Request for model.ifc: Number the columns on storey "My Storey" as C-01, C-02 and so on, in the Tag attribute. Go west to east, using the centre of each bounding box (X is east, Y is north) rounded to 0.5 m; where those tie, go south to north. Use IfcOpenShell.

First a look at what the model holds.

```python
import ifcopenshell
import ifcopenshell.util.element
import ifcopenshell.util.placement

model = ifcopenshell.open("model.ifc")
print(model.schema)
storey = next(s for s in model.by_type("IfcBuildingStorey") if s.Name == "My Storey")
columns = [e for e in ifcopenshell.util.element.get_decomposition(storey) if e.is_a("IfcColumn")]
for e in sorted(columns, key=lambda e: e.id()):
    origin = ifcopenshell.util.placement.get_local_placement(e.ObjectPlacement)[:3, 3]
    print(e.id(), e.Tag, e.Name, origin.round(2) + 0.0, sep=" | ")
```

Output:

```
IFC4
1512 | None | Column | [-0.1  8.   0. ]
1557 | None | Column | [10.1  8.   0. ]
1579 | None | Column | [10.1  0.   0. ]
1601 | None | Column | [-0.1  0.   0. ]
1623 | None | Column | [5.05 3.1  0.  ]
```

```python
import ifcopenshell
import ifcopenshell.geom
import ifcopenshell.util.element
import ifcopenshell.util.shape

model = ifcopenshell.open("model.ifc")
settings = ifcopenshell.geom.settings()
settings.set("use-world-coords", True)


def centre(element):
    shape = ifcopenshell.geom.create_shape(settings, element)
    return ifcopenshell.util.shape.get_bbox_centroid(shape.geometry)


storey = next(s for s in model.by_type("IfcBuildingStorey") if s.Name == "My Storey")
columns = [e for e in ifcopenshell.util.element.get_decomposition(storey) if e.is_a("IfcColumn")]

# Insertion points can sit at a corner or the storey origin, so sort by the geometry (in metres).
centres = {e: centre(e) for e in columns}
columns.sort(key=lambda e: (round(centres[e][0] / 0.5), centres[e][1]))

for i, e in enumerate(columns, start=1):
    number = f"C-{i:02d}"
    e.Tag = number
    print(e.id(), number)

model.write("model_rev.ifc")
```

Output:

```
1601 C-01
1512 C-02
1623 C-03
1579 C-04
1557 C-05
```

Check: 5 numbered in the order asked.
